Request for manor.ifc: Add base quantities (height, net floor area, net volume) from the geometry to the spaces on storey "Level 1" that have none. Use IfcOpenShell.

First a look at what the model holds.

```python
import ifcopenshell
import ifcopenshell.util.element
import ifcopenshell.util.unit

model = ifcopenshell.open("manor.ifc")
print(model.schema)
for unit_type in ("LENGTHUNIT", "AREAUNIT", "VOLUMEUNIT"):
    print(unit_type, ifcopenshell.util.unit.calculate_unit_scale(model, unit_type))
storey = next(s for s in model.by_type("IfcBuildingStorey") if s.Name == "Level 1")
spaces = [e for e in ifcopenshell.util.element.get_decomposition(storey) if e.is_a("IfcSpace")]
for e in sorted(spaces, key=lambda e: e.id()):
    print(e.id(), e.is_a(), e.Name, list(ifcopenshell.util.element.get_psets(e, qtos_only=True)), sep=" | ")
```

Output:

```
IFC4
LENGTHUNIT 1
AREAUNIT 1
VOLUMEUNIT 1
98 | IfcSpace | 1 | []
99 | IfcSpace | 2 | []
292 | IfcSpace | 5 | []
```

```python
import ifcopenshell
import ifcopenshell.api.pset
import ifcopenshell.geom
import ifcopenshell.util.element
import ifcopenshell.util.shape
import ifcopenshell.util.unit

model = ifcopenshell.open("manor.ifc")
unit_scale = ifcopenshell.util.unit.calculate_unit_scale(model)
area_scale = ifcopenshell.util.unit.calculate_unit_scale(model, "AREAUNIT")
volume_scale = ifcopenshell.util.unit.calculate_unit_scale(model, "VOLUMEUNIT")
settings = ifcopenshell.geom.settings()

storey = next(s for s in model.by_type("IfcBuildingStorey") if s.Name == "Level 1")
spaces = [e for e in ifcopenshell.util.element.get_decomposition(storey) if e.is_a("IfcSpace")]

for e in sorted(spaces, key=lambda e: e.id()):
    if ifcopenshell.util.element.get_psets(e, qtos_only=True, should_inherit=False):
        continue
    # Geometry comes back in metres, in the element's own axes.
    shape = ifcopenshell.geom.create_shape(settings, e)
    values = {
        "Height": ifcopenshell.util.shape.get_z(shape.geometry) / unit_scale,
        "NetFloorArea": ifcopenshell.util.shape.get_footprint_area(shape.geometry) / area_scale,
        "NetVolume": ifcopenshell.util.shape.get_volume(shape.geometry) / volume_scale,
    }
    qto = ifcopenshell.api.pset.add_qto(model, product=e, name="Qto_SpaceBaseQuantities")
    ifcopenshell.api.pset.edit_qto(model, qto=qto, properties=values)
    print(e.id(), {k: round(v, 3) for k, v in values.items()})

model.write("manor_updated.ifc")
```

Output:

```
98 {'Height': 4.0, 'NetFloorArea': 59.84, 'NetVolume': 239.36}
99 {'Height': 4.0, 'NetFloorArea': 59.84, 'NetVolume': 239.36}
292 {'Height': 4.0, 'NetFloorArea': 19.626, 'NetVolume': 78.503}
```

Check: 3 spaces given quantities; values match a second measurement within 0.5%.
